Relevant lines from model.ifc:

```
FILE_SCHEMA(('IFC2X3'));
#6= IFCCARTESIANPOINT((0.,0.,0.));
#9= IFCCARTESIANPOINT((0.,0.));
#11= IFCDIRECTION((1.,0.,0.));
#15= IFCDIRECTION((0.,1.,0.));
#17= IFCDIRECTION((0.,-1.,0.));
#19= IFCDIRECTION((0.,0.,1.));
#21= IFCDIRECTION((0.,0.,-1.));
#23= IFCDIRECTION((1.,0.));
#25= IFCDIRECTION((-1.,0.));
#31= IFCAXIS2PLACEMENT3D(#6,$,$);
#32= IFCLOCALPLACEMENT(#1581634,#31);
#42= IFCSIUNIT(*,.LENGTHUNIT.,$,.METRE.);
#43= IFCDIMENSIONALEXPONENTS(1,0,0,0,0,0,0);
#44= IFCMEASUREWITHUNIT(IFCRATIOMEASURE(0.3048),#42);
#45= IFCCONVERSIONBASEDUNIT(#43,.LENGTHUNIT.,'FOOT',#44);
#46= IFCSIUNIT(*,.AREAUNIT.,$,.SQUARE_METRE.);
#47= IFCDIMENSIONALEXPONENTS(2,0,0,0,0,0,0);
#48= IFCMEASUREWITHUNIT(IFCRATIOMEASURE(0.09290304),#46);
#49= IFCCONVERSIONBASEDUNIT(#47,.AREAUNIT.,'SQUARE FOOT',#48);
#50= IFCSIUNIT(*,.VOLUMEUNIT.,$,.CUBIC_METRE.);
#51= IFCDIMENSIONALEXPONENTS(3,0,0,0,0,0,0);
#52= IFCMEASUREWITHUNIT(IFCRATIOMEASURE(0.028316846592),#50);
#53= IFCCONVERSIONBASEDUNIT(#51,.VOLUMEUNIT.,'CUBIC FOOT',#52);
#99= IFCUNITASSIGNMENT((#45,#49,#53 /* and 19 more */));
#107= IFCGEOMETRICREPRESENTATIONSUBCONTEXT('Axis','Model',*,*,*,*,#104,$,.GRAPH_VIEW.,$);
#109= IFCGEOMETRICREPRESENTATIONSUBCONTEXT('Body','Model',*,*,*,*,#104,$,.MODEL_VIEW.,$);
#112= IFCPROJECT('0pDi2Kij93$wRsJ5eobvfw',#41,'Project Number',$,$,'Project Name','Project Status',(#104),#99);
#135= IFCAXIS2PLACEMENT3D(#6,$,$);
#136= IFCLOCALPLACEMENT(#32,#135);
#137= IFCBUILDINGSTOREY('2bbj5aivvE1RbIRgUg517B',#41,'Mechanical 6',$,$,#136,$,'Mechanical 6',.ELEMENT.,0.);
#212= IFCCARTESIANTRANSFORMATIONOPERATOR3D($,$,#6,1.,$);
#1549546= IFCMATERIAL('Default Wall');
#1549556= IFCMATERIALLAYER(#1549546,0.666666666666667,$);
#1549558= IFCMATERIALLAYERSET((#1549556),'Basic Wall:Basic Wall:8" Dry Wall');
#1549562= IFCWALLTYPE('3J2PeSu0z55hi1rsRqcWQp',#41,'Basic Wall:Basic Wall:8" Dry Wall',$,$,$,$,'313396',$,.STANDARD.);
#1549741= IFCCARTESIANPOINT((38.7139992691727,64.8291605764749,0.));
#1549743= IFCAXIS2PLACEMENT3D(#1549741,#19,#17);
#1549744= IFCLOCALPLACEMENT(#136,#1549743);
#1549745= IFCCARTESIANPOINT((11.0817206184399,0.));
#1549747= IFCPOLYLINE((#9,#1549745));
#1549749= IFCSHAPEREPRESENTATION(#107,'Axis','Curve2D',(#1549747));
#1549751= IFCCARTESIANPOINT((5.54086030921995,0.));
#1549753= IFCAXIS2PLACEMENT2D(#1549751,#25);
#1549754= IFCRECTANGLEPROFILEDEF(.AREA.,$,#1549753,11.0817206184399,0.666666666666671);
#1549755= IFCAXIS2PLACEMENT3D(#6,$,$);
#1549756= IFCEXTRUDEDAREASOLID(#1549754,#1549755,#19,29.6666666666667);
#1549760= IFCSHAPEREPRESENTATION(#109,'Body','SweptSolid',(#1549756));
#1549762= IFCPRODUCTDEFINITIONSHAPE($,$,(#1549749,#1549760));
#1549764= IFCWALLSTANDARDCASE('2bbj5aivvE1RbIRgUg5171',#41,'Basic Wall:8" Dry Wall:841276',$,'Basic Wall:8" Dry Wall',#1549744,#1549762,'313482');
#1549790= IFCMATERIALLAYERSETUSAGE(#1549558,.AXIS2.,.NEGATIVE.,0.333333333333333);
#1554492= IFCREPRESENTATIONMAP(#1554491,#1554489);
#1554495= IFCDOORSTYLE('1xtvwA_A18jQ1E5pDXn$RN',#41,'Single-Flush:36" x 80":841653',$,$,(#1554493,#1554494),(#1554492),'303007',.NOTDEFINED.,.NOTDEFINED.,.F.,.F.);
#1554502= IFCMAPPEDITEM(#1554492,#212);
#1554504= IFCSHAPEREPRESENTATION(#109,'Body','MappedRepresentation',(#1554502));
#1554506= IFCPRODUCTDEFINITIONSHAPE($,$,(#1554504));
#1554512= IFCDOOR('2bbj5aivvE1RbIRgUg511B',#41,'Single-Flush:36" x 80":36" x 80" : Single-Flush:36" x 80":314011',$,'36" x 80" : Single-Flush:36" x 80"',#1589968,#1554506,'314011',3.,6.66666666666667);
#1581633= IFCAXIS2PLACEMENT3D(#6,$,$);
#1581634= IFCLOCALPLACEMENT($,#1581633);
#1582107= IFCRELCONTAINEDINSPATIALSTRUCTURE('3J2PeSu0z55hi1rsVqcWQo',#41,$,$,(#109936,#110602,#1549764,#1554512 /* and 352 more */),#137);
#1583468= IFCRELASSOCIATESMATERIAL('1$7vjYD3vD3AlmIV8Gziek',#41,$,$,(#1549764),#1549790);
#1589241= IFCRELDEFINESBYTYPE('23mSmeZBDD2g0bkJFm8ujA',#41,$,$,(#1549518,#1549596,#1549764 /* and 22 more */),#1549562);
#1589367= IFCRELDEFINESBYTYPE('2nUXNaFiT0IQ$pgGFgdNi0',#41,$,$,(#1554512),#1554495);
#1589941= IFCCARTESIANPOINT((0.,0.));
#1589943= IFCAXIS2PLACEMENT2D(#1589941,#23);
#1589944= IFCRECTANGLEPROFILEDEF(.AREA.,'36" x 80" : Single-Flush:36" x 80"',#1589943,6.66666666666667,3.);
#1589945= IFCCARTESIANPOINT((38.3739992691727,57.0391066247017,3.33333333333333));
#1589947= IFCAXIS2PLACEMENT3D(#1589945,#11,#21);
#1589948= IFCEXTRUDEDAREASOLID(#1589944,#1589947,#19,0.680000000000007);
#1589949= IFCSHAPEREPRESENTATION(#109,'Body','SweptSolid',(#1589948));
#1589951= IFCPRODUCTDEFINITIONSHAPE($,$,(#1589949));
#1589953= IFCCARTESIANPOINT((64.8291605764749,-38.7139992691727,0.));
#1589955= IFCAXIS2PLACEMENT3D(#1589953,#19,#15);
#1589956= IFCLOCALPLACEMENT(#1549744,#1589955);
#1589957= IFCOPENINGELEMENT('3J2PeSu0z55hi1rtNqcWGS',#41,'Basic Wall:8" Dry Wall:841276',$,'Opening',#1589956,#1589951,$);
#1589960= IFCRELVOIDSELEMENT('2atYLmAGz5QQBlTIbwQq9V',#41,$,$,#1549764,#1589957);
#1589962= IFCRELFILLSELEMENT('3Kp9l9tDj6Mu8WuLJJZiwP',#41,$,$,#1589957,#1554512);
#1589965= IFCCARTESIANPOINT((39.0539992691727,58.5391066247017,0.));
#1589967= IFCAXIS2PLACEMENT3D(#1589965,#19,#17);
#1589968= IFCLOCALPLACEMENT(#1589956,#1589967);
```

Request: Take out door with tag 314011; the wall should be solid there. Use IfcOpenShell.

```python
import ifcopenshell
import ifcopenshell.api.feature
import ifcopenshell.api.root
import ifcopenshell.geom
import ifcopenshell.util.shape

model = ifcopenshell.open("model.ifc")
settings = ifcopenshell.geom.settings()


def volume(element):
    """Net volume in cubic metres, openings subtracted."""
    shape = ifcopenshell.geom.create_shape(settings, element)
    return ifcopenshell.util.shape.get_volume(shape.geometry)


door = model.by_id(1554512)
opening = door.FillsVoids[0].RelatingOpeningElement
wall = opening.VoidsElements[0].RelatingBuildingElement
before = volume(wall)

ifcopenshell.api.root.remove_product(model, product=door)
ifcopenshell.api.feature.remove_feature(model, feature=opening)

after = volume(wall)

print(f"wall volume {before:.3f} -> {after:.3f} m3")

model.write("model_rev.ifc")
```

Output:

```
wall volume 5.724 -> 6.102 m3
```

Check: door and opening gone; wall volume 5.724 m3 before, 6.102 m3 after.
